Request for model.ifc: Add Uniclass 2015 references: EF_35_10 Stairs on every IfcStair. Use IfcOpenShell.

First a look at what the model holds.

```python
import ifcopenshell

model = ifcopenshell.open("model.ifc")
print(model.schema)
print("classifications:", [c.Name for c in model.by_type("IfcClassification")])
for ifc_class in ("IfcDoor", "IfcRoof", "IfcStair", "IfcWall", "IfcWindow"):
    print(ifc_class, len(model.by_type(ifc_class)))
```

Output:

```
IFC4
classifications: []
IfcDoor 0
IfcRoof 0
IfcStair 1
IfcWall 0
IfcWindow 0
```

```python
import ifcopenshell
import ifcopenshell.api.classification

model = ifcopenshell.open("model.ifc")

system = ifcopenshell.api.classification.add_classification(model, classification="Uniclass 2015")

codes = {
    "IfcStair": ("EF_35_10", "Stairs"),
}
for ifc_class, (code, name) in codes.items():
    products = model.by_type(ifc_class)
    ifcopenshell.api.classification.add_reference(
        model, products=products, classification=system, identification=code, name=name
    )
    print(code, len(products))

model.write("model_updated.ifc")
```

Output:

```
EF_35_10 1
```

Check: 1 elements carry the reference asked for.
